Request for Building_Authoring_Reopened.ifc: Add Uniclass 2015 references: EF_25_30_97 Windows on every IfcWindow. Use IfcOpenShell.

First a look at what the model holds.

```python
import ifcopenshell

model = ifcopenshell.open("Building_Authoring_Reopened.ifc")
print(model.schema)
print("classifications:", [c.Name for c in model.by_type("IfcClassification")])
for ifc_class in ("IfcDoor", "IfcRoof", "IfcStair", "IfcWall", "IfcWindow"):
    print(ifc_class, len(model.by_type(ifc_class)))
```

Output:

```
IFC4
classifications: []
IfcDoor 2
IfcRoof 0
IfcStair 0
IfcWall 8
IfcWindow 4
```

```python
import ifcopenshell
import ifcopenshell.api.classification

model = ifcopenshell.open("Building_Authoring_Reopened.ifc")

system = ifcopenshell.api.classification.add_classification(model, classification="Uniclass 2015")

codes = {
    "IfcWindow": ("EF_25_30_97", "Windows"),
}
for ifc_class, (code, name) in codes.items():
    products = model.by_type(ifc_class)
    ifcopenshell.api.classification.add_reference(
        model, products=products, classification=system, identification=code, name=name
    )
    print(code, len(products))

model.write("Building_Authoring_Reopened_rev.ifc")
```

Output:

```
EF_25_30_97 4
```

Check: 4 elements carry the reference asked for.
